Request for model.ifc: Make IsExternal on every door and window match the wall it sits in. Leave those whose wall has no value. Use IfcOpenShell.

First a look at what the model holds.

```python
import ifcopenshell
import ifcopenshell.util.element

model = ifcopenshell.open("model.ifc")
print(model.schema)
seen = {}
for e in model.by_type("IfcDoor") + model.by_type("IfcWindow"):
    if not e.FillsVoids:
        continue
    host = e.FillsVoids[0].RelatingOpeningElement.VoidsElements[0].RelatingBuildingElement
    own = ifcopenshell.util.element.get_pset(e, f"Pset_{e.is_a()[3:].removesuffix('StandardCase')}Common", "IsExternal")
    wall = ifcopenshell.util.element.get_pset(host, "Pset_WallCommon", "IsExternal")
    seen[e.is_a(), own, wall] = seen.get((e.is_a(), own, wall), 0) + 1
for (cls, own, wall), count in sorted(seen.items(), key=str):
    print(count, cls, "IsExternal:", own, "| host wall:", wall)
```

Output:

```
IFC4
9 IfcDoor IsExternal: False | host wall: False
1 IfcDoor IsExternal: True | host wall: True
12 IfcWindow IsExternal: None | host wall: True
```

```python
import ifcopenshell
import ifcopenshell.api.pset
import ifcopenshell.util.element

model = ifcopenshell.open("model.ifc")

count = 0
for ifc_class, pset_name in (("IfcDoor", "Pset_DoorCommon"), ("IfcWindow", "Pset_WindowCommon")):
    for e in model.by_type(ifc_class):
        if not e.FillsVoids:
            continue
        host = e.FillsVoids[0].RelatingOpeningElement.VoidsElements[0].RelatingBuildingElement
        external = ifcopenshell.util.element.get_pset(host, "Pset_WallCommon", "IsExternal")
        if external is None or ifcopenshell.util.element.get_pset(e, pset_name, "IsExternal") == external:
            continue
        pset = ifcopenshell.api.pset.add_pset(model, product=e, name=pset_name)
        ifcopenshell.api.pset.edit_pset(model, pset=pset, properties={"IsExternal": external})
        count += 1

print(count, "updated")

model.write("model_updated.ifc")
```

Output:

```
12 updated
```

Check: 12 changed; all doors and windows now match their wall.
